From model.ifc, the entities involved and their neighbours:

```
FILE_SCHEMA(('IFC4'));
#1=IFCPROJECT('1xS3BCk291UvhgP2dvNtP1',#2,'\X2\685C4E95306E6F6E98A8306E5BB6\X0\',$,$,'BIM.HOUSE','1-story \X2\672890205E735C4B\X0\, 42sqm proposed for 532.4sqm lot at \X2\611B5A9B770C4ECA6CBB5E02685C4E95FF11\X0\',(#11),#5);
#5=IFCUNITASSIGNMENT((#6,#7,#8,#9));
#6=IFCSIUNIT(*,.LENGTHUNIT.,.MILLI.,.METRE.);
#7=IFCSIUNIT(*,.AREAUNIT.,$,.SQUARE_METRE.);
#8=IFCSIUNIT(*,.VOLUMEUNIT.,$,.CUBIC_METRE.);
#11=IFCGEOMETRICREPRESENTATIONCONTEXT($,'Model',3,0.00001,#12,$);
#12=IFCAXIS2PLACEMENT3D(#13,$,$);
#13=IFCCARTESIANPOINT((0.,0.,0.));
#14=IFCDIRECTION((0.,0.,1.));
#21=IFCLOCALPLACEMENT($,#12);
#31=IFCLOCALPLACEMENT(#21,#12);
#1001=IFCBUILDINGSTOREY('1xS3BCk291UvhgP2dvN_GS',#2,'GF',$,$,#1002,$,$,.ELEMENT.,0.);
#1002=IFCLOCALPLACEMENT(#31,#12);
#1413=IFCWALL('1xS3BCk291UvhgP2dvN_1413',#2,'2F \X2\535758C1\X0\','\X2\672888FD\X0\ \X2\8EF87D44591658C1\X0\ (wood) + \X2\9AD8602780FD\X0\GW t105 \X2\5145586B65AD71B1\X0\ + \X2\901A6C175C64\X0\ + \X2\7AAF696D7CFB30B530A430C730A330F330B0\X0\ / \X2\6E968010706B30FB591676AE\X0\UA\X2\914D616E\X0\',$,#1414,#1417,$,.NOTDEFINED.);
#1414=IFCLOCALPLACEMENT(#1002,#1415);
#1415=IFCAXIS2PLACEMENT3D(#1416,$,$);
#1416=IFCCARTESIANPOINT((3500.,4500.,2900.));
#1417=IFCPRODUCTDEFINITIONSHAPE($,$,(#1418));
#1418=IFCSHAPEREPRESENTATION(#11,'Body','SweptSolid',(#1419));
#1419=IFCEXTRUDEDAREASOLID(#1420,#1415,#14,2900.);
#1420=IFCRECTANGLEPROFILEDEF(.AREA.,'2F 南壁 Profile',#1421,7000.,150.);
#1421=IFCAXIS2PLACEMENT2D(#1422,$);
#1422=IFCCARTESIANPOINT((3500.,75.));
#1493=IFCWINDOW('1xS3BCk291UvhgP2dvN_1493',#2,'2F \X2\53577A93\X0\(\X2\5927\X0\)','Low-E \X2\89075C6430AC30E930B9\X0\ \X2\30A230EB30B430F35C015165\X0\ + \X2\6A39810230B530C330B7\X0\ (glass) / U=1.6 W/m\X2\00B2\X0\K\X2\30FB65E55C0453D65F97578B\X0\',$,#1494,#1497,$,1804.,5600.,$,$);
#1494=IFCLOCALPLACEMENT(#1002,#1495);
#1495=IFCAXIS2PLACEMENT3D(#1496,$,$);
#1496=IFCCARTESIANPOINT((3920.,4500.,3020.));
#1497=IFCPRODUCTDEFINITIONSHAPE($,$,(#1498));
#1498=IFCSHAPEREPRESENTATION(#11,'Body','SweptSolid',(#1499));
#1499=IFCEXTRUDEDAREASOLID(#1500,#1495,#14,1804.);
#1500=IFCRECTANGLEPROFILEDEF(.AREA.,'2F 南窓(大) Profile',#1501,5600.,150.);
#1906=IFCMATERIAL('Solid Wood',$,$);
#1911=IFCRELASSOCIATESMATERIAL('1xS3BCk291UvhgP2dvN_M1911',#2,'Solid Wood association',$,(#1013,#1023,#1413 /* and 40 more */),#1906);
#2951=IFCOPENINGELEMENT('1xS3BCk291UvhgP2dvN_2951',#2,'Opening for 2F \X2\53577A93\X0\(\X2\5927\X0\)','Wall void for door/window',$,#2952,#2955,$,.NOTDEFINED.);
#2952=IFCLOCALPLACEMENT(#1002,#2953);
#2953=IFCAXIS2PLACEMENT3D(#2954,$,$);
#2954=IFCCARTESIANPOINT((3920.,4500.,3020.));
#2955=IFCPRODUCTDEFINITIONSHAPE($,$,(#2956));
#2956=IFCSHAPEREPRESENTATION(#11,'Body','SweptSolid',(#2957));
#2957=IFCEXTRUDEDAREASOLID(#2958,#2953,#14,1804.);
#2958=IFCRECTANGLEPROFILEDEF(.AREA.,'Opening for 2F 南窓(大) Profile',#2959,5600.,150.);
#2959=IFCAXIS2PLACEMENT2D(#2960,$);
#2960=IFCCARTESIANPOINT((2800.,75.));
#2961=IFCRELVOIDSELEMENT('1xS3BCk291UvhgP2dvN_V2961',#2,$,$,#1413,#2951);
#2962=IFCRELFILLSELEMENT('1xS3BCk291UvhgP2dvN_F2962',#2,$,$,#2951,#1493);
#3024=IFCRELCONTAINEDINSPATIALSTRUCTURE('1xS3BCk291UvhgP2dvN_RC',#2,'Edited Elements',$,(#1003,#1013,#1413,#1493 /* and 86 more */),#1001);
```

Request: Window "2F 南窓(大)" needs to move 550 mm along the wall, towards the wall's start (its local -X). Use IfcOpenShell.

```python
import ifcopenshell
import ifcopenshell.api.geometry
import ifcopenshell.util.placement

model = ifcopenshell.open("model.ifc")

window = model.by_guid("1xS3BCk291UvhgP2dvN_1493")
opening = window.FillsVoids[0].RelatingOpeningElement
wall = opening.VoidsElements[0].RelatingBuildingElement

wall_matrix = ifcopenshell.util.placement.get_local_placement(wall.ObjectPlacement)
shift = wall_matrix[:3, 0] * -550.0
before = ifcopenshell.util.placement.get_local_placement(window.ObjectPlacement)[:3, 3].copy()

# The window is not placed relative to its opening, so move both.
for product in (opening, window):
    matrix = ifcopenshell.util.placement.get_local_placement(product.ObjectPlacement)
    matrix[:3, 3] += shift
    ifcopenshell.api.geometry.edit_object_placement(model, product=product, matrix=matrix, is_si=False)

after = ifcopenshell.util.placement.get_local_placement(window.ObjectPlacement)[:3, 3]
print("window moved by", (after - before).round(3) + 0.0)

model.write("model_rev.ifc")
```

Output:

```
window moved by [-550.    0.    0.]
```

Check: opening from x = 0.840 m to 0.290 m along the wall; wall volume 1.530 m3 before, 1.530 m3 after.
